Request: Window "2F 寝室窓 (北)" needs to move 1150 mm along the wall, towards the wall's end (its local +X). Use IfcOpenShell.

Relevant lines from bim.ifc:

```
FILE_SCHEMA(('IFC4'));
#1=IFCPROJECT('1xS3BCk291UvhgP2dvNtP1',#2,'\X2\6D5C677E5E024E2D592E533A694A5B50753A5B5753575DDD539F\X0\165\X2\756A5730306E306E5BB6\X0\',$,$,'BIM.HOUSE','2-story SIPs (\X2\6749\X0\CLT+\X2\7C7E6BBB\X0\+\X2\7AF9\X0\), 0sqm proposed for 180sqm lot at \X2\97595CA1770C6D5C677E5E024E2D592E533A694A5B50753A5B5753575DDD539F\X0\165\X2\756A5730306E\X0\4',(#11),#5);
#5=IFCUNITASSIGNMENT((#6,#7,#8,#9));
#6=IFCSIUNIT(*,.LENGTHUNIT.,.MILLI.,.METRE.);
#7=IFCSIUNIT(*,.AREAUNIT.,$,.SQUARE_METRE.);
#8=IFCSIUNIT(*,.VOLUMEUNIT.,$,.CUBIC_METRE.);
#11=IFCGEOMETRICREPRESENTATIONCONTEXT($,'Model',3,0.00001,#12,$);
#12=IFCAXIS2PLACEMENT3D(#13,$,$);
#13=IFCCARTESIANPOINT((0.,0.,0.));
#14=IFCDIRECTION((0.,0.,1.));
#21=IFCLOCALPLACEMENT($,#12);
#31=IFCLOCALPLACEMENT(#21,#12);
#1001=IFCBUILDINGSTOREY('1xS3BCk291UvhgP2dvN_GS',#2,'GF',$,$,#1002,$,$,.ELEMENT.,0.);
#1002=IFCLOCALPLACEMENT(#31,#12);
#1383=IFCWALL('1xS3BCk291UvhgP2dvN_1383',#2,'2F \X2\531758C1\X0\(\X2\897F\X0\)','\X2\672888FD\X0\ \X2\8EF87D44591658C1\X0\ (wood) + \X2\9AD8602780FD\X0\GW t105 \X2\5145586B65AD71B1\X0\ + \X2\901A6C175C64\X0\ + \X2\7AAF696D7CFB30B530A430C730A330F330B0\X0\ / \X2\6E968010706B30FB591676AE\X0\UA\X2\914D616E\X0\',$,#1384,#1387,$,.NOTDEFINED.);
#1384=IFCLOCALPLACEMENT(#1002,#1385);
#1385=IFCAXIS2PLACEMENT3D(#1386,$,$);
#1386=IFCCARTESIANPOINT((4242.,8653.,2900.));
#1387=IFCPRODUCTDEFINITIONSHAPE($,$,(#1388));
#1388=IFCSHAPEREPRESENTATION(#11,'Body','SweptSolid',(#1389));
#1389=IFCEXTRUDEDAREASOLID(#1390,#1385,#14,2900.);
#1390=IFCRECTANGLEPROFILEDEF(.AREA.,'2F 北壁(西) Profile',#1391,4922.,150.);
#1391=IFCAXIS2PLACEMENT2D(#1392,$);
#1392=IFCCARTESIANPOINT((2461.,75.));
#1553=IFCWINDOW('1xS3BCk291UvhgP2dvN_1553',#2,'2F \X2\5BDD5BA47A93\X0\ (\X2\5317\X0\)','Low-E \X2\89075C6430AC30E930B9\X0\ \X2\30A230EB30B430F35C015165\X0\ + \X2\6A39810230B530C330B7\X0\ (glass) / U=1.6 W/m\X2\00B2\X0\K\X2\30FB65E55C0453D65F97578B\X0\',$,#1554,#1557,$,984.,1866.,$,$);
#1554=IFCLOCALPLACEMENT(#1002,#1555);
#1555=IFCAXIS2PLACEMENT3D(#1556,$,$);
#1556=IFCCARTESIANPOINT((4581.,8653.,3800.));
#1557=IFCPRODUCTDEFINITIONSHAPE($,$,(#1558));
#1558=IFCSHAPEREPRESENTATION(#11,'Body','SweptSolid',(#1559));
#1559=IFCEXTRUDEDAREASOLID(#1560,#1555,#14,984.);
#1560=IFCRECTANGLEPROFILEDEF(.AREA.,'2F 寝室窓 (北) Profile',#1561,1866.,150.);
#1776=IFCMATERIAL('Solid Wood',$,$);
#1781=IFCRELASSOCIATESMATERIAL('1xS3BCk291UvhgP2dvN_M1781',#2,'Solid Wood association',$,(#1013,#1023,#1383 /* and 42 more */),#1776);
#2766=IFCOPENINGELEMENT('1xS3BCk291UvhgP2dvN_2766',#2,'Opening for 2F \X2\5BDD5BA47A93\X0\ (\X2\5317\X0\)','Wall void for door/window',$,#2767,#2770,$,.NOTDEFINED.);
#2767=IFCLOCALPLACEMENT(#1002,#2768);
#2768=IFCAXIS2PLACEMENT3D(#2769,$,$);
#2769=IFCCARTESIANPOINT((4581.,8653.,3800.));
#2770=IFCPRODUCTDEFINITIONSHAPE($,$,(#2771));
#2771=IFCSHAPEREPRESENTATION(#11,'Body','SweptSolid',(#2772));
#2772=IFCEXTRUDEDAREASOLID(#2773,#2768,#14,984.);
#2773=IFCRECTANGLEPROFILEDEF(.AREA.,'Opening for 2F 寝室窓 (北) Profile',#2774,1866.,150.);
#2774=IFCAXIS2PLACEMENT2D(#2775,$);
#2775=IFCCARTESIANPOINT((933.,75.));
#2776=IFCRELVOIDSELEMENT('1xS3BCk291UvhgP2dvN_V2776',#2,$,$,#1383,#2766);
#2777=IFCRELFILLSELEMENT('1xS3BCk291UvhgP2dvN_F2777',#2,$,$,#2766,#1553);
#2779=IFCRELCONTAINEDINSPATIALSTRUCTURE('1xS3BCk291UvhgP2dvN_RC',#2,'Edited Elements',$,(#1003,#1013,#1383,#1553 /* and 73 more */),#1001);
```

```python
import ifcopenshell
import ifcopenshell.api.geometry
import ifcopenshell.util.placement
import ifcopenshell.util.unit

model = ifcopenshell.open("bim.ifc")
unit_scale = ifcopenshell.util.unit.calculate_unit_scale(model)

window = model.by_guid("1xS3BCk291UvhgP2dvN_1553")
opening = window.FillsVoids[0].RelatingOpeningElement
wall = opening.VoidsElements[0].RelatingBuildingElement

wall_matrix = ifcopenshell.util.placement.get_local_placement(wall.ObjectPlacement)
shift = wall_matrix[:3, 0] * 1.15 / unit_scale
before = ifcopenshell.util.placement.get_local_placement(window.ObjectPlacement)[:3, 3].copy()

# The window is not placed relative to its opening, so move both.
for product in (opening, window):
    matrix = ifcopenshell.util.placement.get_local_placement(product.ObjectPlacement)
    matrix[:3, 3] += shift
    ifcopenshell.api.geometry.edit_object_placement(model, product=product, matrix=matrix, is_si=False)

after = ifcopenshell.util.placement.get_local_placement(window.ObjectPlacement)[:3, 3]
print("window moved by", (after - before).round(3) + 0.0)

model.write("bim-out.ifc")
```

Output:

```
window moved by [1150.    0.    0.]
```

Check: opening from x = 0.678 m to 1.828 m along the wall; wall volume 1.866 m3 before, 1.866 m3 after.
